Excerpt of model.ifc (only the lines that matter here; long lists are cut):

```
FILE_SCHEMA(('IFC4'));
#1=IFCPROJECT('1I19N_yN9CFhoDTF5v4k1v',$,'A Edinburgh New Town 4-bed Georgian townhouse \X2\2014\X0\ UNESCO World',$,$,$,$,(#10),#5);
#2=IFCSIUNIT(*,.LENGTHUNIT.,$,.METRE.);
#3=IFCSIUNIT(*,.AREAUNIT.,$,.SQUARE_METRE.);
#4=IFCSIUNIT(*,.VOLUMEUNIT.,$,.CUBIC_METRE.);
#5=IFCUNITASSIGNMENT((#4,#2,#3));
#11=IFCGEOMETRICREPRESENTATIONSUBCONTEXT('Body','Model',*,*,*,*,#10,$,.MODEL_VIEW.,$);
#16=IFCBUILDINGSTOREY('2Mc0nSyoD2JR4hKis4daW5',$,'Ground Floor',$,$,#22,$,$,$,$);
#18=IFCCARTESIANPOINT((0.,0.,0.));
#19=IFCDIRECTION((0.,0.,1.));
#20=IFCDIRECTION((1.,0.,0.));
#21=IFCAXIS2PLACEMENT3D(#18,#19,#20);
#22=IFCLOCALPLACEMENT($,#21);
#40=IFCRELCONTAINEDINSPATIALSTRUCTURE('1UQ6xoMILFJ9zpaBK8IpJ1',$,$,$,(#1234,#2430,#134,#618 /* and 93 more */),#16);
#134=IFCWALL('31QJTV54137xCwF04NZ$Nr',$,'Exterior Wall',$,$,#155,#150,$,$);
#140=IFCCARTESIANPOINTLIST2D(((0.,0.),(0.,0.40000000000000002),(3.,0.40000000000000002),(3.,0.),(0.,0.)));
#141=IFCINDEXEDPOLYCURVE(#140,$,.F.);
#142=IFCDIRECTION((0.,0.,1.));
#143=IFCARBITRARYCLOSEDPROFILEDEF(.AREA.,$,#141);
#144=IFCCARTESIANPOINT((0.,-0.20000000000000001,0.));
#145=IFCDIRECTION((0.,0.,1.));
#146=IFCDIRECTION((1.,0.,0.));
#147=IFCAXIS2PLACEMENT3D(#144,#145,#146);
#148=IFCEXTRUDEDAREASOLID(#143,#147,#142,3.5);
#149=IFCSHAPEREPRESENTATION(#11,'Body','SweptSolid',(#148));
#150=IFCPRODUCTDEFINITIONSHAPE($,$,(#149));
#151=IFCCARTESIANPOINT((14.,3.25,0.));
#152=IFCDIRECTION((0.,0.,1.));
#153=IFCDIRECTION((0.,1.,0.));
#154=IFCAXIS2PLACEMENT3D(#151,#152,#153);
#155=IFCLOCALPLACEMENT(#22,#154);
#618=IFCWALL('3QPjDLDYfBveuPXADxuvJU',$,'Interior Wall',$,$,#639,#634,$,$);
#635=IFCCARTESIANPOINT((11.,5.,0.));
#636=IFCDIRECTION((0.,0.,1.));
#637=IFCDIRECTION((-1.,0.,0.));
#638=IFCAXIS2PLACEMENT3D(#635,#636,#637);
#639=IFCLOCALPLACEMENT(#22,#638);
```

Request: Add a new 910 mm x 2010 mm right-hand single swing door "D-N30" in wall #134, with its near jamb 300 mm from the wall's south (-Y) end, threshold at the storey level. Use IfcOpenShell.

```python
import numpy as np
import ifcopenshell
import ifcopenshell.api.feature
import ifcopenshell.api.geometry
import ifcopenshell.api.root
import ifcopenshell.api.spatial
import ifcopenshell.geom
import ifcopenshell.util.element
import ifcopenshell.util.placement
import ifcopenshell.util.representation
import ifcopenshell.util.shape
import ifcopenshell.util.unit

model = ifcopenshell.open("model.ifc")
unit_scale = ifcopenshell.util.unit.calculate_unit_scale(model)
settings = ifcopenshell.geom.settings()


def volume(element):
    """Net volume in cubic metres, openings subtracted."""
    shape = ifcopenshell.geom.create_shape(settings, element)
    return ifcopenshell.util.shape.get_volume(shape.geometry)


wall = model.by_id(134)
storey = ifcopenshell.util.element.get_container(wall, ifc_class="IfcBuildingStorey")
context = ifcopenshell.util.representation.get_context(model, "Model", "Body", "MODEL_VIEW")
before = volume(wall)

width, height, from_end, sill = 0.91, 2.01, 0.3, 0.0  # metres

# The wall runs along its own X axis, and the end named is its -X end.
wall_shape = ifcopenshell.geom.create_shape(settings, wall)
x, y, z = ifcopenshell.util.shape.get_vertices(wall_shape.geometry).T
start = x.min() + from_end
face, thickness = float(y.min()), float(y.max() - y.min())
wall_matrix = ifcopenshell.util.placement.get_local_placement(wall.ObjectPlacement)
level = ifcopenshell.util.placement.get_local_placement(storey.ObjectPlacement)[2, 3]


def in_wall(x, y):
    """Placement at x, y metres in the wall's axes, at sill height."""
    matrix = wall_matrix.copy()
    matrix[:, 3] = wall_matrix @ np.array([x / unit_scale, y / unit_scale, 0.0, 1.0])
    matrix[2, 3] = level + sill / unit_scale
    return matrix


# Opening: a box that overshoots both wall faces by 50 mm.
opening = ifcopenshell.api.root.create_entity(model, ifc_class="IfcOpeningElement", predefined_type="OPENING")
box = ifcopenshell.api.geometry.add_wall_representation(
    model, context=context, length=width, height=height, thickness=thickness + 0.1
)
ifcopenshell.api.geometry.assign_representation(model, product=opening, representation=box)
ifcopenshell.api.geometry.edit_object_placement(model, product=opening, matrix=in_wall(start, face - 0.05), is_si=False)
ifcopenshell.api.feature.add_feature(model, feature=opening, element=wall)

door = ifcopenshell.api.root.create_entity(model, ifc_class="IfcDoor", name="D-N30", predefined_type="DOOR")
door.OverallWidth, door.OverallHeight = width / unit_scale, height / unit_scale
door.OperationType = "SINGLE_SWING_RIGHT"
body = ifcopenshell.api.geometry.add_door_representation(
    model,
    context=context,
    overall_width=door.OverallWidth,
    overall_height=door.OverallHeight,
    operation_type="SINGLE_SWING_RIGHT",
    lining_properties={"LiningDepth": thickness / unit_scale, "ThresholdDepth": thickness / unit_scale},
)
ifcopenshell.api.geometry.assign_representation(model, product=door, representation=body)
ifcopenshell.api.spatial.assign_container(model, products=[door], relating_structure=storey)
ifcopenshell.api.feature.add_filling(model, opening=opening, element=door)

# The lining spans the wall, so the door starts at the wall face.
ifcopenshell.api.geometry.edit_object_placement(model, product=door, matrix=in_wall(start, face), is_si=False)

after = volume(wall)

print(f"wall volume {before:.3f} -> {after:.3f} m3")

model.write("model_edited.ifc")
```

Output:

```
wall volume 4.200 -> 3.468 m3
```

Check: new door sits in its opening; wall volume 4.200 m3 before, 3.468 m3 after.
